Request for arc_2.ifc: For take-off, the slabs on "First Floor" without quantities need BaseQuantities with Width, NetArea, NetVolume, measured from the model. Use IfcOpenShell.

First a look at what the model holds.

```python
import ifcopenshell
import ifcopenshell.util.element
import ifcopenshell.util.unit

model = ifcopenshell.open("arc_2.ifc")
print(model.schema)
for unit_type in ("LENGTHUNIT", "AREAUNIT", "VOLUMEUNIT"):
    print(unit_type, ifcopenshell.util.unit.calculate_unit_scale(model, unit_type))
storey = next(s for s in model.by_type("IfcBuildingStorey") if s.Name == "First Floor")
slabs = [e for e in ifcopenshell.util.element.get_decomposition(storey) if e.is_a("IfcSlab")]
for e in sorted(slabs, key=lambda e: e.id()):
    print(e.id(), e.is_a(), e.Name, list(ifcopenshell.util.element.get_psets(e, qtos_only=True)), sep=" | ")
```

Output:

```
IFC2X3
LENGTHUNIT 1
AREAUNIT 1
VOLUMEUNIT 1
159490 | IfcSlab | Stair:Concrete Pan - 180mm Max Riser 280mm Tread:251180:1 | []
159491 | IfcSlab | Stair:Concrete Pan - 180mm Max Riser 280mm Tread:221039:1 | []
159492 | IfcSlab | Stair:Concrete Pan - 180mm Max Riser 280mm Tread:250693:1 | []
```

```python
import ifcopenshell
import ifcopenshell.api.pset
import ifcopenshell.geom
import ifcopenshell.util.element
import ifcopenshell.util.shape
import ifcopenshell.util.unit

model = ifcopenshell.open("arc_2.ifc")
unit_scale = ifcopenshell.util.unit.calculate_unit_scale(model)
area_scale = ifcopenshell.util.unit.calculate_unit_scale(model, "AREAUNIT")
volume_scale = ifcopenshell.util.unit.calculate_unit_scale(model, "VOLUMEUNIT")
settings = ifcopenshell.geom.settings()

storey = next(s for s in model.by_type("IfcBuildingStorey") if s.Name == "First Floor")
slabs = [e for e in ifcopenshell.util.element.get_decomposition(storey) if e.is_a("IfcSlab")]

for e in sorted(slabs, key=lambda e: e.id()):
    if ifcopenshell.util.element.get_psets(e, qtos_only=True, should_inherit=False):
        continue
    # Geometry comes back in metres, in the element's own axes.
    shape = ifcopenshell.geom.create_shape(settings, e)
    values = {
        "Width": ifcopenshell.util.shape.get_z(shape.geometry) / unit_scale,
        "NetArea": ifcopenshell.util.shape.get_footprint_area(shape.geometry) / area_scale,
        "NetVolume": ifcopenshell.util.shape.get_volume(shape.geometry) / volume_scale,
    }
    qto = ifcopenshell.api.pset.add_qto(model, product=e, name="BaseQuantities")
    ifcopenshell.api.pset.edit_qto(model, qto=qto, properties=values)
    print(e.id(), {k: round(v, 3) for k, v in values.items()})

model.write("arc_2_rev.ifc")
```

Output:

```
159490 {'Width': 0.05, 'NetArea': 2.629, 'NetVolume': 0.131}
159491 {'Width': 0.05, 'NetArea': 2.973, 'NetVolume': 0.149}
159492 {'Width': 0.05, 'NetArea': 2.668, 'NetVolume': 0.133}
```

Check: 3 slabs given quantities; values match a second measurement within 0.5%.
